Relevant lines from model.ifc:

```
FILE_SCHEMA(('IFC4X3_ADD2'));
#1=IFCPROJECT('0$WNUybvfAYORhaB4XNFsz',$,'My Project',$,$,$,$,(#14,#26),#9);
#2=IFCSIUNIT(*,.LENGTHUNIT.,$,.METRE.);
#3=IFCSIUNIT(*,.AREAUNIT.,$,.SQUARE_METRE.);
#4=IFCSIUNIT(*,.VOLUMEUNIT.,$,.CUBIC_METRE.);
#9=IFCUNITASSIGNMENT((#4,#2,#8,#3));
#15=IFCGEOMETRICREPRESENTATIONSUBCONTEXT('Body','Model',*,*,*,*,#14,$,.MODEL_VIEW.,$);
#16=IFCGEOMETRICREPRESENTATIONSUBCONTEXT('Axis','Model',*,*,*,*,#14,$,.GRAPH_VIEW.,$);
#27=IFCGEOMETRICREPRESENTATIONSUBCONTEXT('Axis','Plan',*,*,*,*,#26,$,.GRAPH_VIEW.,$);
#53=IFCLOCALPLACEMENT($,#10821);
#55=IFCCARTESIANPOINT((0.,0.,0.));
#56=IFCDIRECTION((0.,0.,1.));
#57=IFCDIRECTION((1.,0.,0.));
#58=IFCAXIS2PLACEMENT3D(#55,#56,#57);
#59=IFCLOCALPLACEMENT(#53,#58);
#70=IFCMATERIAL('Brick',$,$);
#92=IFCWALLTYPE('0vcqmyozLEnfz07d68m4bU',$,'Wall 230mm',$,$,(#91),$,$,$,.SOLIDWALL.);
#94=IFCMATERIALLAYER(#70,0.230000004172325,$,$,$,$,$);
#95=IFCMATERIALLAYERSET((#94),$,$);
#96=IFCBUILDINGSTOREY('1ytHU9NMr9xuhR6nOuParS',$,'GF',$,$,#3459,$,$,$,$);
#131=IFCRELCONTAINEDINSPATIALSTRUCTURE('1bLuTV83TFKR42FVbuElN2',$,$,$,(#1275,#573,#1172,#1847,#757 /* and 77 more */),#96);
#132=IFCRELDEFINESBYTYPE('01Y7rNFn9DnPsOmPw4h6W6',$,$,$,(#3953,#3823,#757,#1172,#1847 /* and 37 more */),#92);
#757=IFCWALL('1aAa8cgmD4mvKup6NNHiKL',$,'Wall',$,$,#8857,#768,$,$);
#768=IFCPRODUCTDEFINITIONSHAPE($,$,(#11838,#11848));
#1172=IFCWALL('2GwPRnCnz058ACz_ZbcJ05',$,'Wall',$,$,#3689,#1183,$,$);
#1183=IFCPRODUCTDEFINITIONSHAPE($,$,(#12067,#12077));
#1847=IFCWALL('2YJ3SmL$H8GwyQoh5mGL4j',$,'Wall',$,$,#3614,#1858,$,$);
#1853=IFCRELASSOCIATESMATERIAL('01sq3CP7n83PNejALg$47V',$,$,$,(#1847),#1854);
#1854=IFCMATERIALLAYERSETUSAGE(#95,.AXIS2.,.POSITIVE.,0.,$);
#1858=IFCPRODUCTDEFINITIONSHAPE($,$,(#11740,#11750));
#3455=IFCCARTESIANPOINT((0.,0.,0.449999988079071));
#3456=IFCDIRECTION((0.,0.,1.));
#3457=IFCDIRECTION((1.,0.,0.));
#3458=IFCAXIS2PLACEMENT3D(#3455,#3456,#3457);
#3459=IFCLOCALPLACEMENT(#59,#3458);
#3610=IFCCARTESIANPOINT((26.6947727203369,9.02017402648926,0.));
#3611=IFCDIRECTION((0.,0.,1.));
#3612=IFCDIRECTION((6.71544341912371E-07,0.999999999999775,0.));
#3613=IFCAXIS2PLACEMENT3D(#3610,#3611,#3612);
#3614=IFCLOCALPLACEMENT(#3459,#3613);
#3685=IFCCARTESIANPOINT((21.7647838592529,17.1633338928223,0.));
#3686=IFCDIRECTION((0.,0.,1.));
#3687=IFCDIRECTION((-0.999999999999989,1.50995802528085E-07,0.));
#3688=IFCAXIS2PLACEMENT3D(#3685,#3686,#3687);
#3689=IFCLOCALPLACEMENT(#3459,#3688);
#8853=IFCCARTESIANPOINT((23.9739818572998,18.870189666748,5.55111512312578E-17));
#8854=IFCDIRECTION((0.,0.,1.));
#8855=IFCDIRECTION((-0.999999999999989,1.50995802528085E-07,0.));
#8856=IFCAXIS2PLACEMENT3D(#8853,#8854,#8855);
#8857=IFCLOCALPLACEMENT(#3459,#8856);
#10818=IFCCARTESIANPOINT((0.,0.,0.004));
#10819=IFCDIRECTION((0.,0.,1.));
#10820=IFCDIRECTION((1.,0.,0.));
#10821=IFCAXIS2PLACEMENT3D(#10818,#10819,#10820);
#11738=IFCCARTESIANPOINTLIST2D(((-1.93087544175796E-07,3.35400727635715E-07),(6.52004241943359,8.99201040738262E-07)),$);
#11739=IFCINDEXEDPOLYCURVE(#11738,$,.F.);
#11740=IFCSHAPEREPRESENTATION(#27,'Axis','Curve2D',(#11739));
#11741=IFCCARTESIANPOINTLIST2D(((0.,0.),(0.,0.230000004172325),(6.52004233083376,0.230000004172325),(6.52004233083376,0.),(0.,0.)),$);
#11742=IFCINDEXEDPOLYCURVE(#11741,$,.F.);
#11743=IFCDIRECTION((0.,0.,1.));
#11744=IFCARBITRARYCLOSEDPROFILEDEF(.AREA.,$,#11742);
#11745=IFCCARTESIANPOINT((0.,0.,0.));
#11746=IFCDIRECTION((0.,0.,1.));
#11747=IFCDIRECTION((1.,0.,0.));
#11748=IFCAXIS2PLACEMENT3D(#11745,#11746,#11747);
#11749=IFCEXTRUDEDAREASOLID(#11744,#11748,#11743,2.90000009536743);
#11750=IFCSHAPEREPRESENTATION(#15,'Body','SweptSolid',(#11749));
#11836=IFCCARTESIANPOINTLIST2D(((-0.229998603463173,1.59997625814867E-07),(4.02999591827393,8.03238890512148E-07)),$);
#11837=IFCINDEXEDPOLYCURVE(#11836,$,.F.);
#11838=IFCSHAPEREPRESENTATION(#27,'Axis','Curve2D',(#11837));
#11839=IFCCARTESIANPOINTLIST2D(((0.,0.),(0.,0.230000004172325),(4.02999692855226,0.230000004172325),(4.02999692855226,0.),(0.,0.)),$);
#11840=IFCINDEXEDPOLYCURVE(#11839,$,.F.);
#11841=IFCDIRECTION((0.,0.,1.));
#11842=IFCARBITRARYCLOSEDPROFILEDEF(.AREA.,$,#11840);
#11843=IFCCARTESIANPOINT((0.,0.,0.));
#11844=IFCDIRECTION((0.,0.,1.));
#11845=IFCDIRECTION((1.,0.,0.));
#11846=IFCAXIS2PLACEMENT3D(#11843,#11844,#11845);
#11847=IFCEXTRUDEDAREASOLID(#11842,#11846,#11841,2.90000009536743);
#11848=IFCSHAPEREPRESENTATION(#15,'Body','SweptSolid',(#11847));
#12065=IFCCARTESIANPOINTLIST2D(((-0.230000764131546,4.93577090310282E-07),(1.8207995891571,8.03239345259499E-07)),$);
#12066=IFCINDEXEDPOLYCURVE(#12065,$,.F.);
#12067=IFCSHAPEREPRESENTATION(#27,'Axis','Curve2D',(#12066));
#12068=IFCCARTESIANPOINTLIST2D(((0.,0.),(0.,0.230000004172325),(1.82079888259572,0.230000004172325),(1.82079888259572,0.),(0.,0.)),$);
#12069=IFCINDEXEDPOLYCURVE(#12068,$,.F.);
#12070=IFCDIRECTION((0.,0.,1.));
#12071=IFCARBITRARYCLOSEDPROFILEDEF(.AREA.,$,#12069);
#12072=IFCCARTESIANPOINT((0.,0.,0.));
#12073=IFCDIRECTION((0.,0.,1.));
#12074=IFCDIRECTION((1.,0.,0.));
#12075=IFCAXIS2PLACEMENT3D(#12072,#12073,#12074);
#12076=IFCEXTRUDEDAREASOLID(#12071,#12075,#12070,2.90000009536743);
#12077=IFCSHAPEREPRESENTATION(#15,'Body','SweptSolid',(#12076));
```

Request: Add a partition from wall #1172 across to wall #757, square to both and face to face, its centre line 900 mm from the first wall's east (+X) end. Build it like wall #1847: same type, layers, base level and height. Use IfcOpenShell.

```python
import numpy as np
import ifcopenshell
import ifcopenshell.api.geometry
import ifcopenshell.api.material
import ifcopenshell.api.pset
import ifcopenshell.api.root
import ifcopenshell.api.spatial
import ifcopenshell.api.type
import ifcopenshell.geom
import ifcopenshell.util.element
import ifcopenshell.util.placement
import ifcopenshell.util.representation
import ifcopenshell.util.shape
import ifcopenshell.util.unit

model = ifcopenshell.open("model.ifc")
unit_scale = ifcopenshell.util.unit.calculate_unit_scale(model)
settings = ifcopenshell.geom.settings()
settings.set("use-world-coords", True)

start_wall = model.by_guid("2GwPRnCnz058ACz_ZbcJ05")
end_wall = model.by_id(757)
like = model.by_guid("2YJ3SmL$H8GwyQoh5mGL4j")
matrix = ifcopenshell.util.placement.get_local_placement(start_wall.ObjectPlacement)
matrix[:3, 3] *= unit_scale


def extent(element):
    """Bounding box in the first wall's axes, in metres."""
    shape = ifcopenshell.geom.create_shape(settings, element)
    points = (ifcopenshell.util.shape.get_vertices(shape.geometry) - matrix[:3, 3]) @ matrix[:3, :3]
    return points.min(axis=0), points.max(axis=0)


y_start = extent(start_wall)[0][1]
y_end = extent(end_wall)[1][1]
like_min, like_max = extent(like)
length, height = float(abs(y_end - y_start)), float(like_max[2] - like_min[2])
layer_set = ifcopenshell.util.element.get_material(like, should_skip_usage=True)
thickness = sum(layer.LayerThickness for layer in layer_set.MaterialLayers) * unit_scale

wall = ifcopenshell.api.root.create_entity(model, ifc_class="IfcWall", name="New partition")
storey = ifcopenshell.util.element.get_container(like)
ifcopenshell.api.spatial.assign_container(model, products=[wall], relating_structure=storey)
ifcopenshell.api.type.assign_type(
    model, related_objects=[wall], relating_type=ifcopenshell.util.element.get_type(like), should_map_representations=False
)
rel = ifcopenshell.api.material.assign_material(
    model, products=[wall], type="IfcMaterialLayerSetUsage", material=layer_set
)
rel.RelatingMaterial.OffsetFromReferenceLine = -thickness / 2 / unit_scale
pset = ifcopenshell.api.pset.add_pset(model, product=wall, name="Pset_WallCommon")
ifcopenshell.api.pset.edit_pset(model, pset=pset, properties={"IsExternal": False, "LoadBearing": False})

# The axis runs down the middle of the wall.
axis = ifcopenshell.api.geometry.add_axis_representation(
    model, context=ifcopenshell.util.representation.get_context(model, "Model", "Axis"), axis=[(0.0, 0.0), (length, 0.0)]
)
body = ifcopenshell.api.geometry.add_wall_representation(
    model,
    context=ifcopenshell.util.representation.get_context(model, "Model", "Body", "MODEL_VIEW"),
    length=length,
    height=height,
    thickness=thickness,
    offset=-thickness / 2,
)
for representation in (axis, body):
    ifcopenshell.api.geometry.assign_representation(model, product=wall, representation=representation)

placement = matrix @ ifcopenshell.util.placement.rotation(-90, "Z")
placement[:, 3] = matrix @ np.array([extent(start_wall)[0][0] + 0.9, y_start, like_min[2], 1.0])
ifcopenshell.api.geometry.edit_object_placement(model, product=wall, matrix=placement)

print(f"partition {length:.3f} m long, {height:.3f} m high, {thickness:.3f} m thick")

model.write("model_updated.ifc")
```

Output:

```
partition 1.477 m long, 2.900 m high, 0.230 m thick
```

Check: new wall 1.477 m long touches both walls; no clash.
